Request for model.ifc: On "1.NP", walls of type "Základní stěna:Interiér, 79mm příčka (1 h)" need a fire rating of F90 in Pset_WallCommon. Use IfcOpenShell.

First a look at what the model holds.

```python
import ifcopenshell
import ifcopenshell.util.element

model = ifcopenshell.open("model.ifc")
print(model.schema)
storey = next(s for s in model.by_type("IfcBuildingStorey") if s.Name == "1.NP")
walls = [e for e in ifcopenshell.util.element.get_decomposition(storey) if e.is_a("IfcWall")]
seen = {}
for e in walls:
    element_type = ifcopenshell.util.element.get_type(e)
    key = (element_type.Name if element_type != e and element_type else None, ifcopenshell.util.element.get_pset(e, "Pset_WallCommon", "FireRating"))
    seen[key] = seen.get(key, 0) + 1
for (name, value), count in sorted(seen.items(), key=str):
    print(count, "x", name, "|", value)
```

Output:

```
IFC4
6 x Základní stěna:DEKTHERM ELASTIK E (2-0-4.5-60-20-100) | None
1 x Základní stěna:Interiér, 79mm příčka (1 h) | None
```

```python
import ifcopenshell
import ifcopenshell.api.pset
import ifcopenshell.util.element

model = ifcopenshell.open("model.ifc")

storey = next(s for s in model.by_type("IfcBuildingStorey") if s.Name == "1.NP")
walls = [e for e in ifcopenshell.util.element.get_decomposition(storey) if e.is_a("IfcWall")]

count = 0
for e in walls:
    element_type = ifcopenshell.util.element.get_type(e)
    if element_type in (None, e) or element_type.Name != "Základní stěna:Interiér, 79mm příčka (1 h)":
        continue
    # add_pset returns the element's existing set when there is one.
    pset = ifcopenshell.api.pset.add_pset(model, product=e, name="Pset_WallCommon")
    ifcopenshell.api.pset.edit_pset(model, pset=pset, properties={"FireRating": "F90"})
    count += 1

print(count, "walls updated")

model.write("model_rev.ifc")
```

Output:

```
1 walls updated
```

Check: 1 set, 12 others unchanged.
